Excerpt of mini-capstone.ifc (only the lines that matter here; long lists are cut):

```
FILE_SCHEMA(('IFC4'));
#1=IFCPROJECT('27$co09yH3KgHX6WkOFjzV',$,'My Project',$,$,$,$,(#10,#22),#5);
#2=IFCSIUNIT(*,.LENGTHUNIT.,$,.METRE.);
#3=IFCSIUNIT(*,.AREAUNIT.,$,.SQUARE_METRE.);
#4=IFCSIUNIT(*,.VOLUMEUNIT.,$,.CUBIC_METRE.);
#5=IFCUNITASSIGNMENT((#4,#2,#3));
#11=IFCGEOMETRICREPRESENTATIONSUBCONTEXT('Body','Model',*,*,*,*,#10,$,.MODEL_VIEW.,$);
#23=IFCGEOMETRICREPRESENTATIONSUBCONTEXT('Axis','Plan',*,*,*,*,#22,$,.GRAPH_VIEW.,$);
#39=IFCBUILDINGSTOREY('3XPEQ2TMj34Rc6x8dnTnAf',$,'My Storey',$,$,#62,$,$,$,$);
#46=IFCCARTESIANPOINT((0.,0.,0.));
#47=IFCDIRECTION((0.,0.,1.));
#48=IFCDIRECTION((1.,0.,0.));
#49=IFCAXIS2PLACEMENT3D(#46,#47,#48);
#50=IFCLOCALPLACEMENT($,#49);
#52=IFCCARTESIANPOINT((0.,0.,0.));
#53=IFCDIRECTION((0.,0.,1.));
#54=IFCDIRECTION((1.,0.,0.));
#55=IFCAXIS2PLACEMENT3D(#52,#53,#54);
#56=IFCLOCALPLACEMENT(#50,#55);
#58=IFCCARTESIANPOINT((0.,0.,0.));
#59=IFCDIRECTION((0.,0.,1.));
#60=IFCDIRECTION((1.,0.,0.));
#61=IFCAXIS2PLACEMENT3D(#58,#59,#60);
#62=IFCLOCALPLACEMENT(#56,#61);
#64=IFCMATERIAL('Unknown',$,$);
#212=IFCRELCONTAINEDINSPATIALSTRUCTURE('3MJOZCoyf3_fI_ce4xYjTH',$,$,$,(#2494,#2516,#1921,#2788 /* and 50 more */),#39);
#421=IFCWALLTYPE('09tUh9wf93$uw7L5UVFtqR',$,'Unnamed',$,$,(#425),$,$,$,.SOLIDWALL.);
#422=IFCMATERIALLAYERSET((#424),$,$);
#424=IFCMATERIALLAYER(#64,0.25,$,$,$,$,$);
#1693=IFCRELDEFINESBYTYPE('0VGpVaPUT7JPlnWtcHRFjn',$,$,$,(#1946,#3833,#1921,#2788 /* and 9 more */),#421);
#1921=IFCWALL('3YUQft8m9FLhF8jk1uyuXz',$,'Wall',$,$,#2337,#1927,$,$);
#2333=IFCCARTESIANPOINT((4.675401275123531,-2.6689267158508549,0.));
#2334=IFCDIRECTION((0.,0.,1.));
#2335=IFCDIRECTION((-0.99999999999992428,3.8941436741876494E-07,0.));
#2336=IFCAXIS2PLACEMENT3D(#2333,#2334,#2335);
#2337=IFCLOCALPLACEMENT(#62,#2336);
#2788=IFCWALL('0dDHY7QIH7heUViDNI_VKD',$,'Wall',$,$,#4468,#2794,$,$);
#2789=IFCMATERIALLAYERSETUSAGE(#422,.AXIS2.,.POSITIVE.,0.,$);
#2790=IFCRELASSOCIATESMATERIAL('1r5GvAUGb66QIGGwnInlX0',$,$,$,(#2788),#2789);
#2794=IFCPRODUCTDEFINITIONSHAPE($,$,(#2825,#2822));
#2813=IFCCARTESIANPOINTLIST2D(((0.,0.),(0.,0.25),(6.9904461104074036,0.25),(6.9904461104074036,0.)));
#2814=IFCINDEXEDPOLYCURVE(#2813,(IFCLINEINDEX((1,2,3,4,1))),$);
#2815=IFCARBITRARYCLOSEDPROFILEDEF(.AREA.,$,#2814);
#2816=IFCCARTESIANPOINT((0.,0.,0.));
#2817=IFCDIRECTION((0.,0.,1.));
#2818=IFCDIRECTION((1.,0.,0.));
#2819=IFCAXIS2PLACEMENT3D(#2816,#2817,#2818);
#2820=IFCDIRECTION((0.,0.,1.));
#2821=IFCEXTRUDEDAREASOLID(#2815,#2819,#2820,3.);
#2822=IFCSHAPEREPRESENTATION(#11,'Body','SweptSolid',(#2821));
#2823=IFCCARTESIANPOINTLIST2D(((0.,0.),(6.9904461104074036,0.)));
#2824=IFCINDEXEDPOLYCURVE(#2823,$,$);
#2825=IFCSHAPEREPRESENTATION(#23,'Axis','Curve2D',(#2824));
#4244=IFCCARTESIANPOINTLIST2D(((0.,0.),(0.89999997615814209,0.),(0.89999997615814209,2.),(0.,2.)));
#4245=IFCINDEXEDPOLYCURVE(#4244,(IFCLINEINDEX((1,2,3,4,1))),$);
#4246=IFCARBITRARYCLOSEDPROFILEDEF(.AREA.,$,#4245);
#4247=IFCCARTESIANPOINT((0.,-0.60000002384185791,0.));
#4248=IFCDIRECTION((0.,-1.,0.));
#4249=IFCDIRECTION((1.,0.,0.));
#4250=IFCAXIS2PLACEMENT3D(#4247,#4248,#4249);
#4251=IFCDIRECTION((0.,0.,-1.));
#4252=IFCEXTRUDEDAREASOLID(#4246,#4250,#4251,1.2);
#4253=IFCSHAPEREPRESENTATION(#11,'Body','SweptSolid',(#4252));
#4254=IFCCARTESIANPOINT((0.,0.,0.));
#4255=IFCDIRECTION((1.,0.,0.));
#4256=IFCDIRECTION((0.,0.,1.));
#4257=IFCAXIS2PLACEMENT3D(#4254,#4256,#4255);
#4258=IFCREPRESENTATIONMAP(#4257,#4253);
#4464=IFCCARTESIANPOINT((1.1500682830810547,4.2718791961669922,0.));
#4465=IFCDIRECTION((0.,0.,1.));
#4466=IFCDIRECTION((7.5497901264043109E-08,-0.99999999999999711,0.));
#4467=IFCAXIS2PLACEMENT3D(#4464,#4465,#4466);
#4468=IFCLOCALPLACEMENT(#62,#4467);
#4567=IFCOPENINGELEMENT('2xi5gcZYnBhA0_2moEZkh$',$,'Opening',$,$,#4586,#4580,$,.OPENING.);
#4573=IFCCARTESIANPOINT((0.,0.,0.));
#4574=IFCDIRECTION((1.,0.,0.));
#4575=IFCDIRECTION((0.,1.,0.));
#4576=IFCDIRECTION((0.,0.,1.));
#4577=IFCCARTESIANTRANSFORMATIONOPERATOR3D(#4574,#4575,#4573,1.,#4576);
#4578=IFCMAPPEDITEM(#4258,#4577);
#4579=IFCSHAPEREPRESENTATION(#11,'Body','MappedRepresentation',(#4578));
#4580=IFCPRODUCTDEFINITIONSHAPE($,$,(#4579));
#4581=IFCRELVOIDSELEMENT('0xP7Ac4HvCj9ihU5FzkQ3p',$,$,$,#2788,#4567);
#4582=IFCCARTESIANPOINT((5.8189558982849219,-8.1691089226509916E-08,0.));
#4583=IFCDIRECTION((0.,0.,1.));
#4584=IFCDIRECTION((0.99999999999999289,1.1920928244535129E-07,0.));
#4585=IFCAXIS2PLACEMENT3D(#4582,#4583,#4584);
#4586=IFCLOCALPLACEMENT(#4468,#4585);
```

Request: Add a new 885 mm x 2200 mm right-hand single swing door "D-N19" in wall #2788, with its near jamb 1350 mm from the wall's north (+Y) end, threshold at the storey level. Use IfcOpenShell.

```python
import numpy as np
import ifcopenshell
import ifcopenshell.api.feature
import ifcopenshell.api.geometry
import ifcopenshell.api.root
import ifcopenshell.api.spatial
import ifcopenshell.geom
import ifcopenshell.util.element
import ifcopenshell.util.placement
import ifcopenshell.util.representation
import ifcopenshell.util.shape
import ifcopenshell.util.unit

model = ifcopenshell.open("mini-capstone.ifc")
unit_scale = ifcopenshell.util.unit.calculate_unit_scale(model)
settings = ifcopenshell.geom.settings()


def volume(element):
    """Net volume in cubic metres, openings subtracted."""
    shape = ifcopenshell.geom.create_shape(settings, element)
    return ifcopenshell.util.shape.get_volume(shape.geometry)


wall = model.by_guid("0dDHY7QIH7heUViDNI_VKD")
storey = ifcopenshell.util.element.get_container(wall, ifc_class="IfcBuildingStorey")
context = ifcopenshell.util.representation.get_context(model, "Model", "Body", "MODEL_VIEW")
before = volume(wall)

width, height, from_end, sill = 0.885, 2.2, 1.35, 0.0  # metres

# The wall runs along its own X axis, and the end named is its -X end.
wall_shape = ifcopenshell.geom.create_shape(settings, wall)
x, y, z = ifcopenshell.util.shape.get_vertices(wall_shape.geometry).T
start = x.min() + from_end
face, thickness = float(y.min()), float(y.max() - y.min())
wall_matrix = ifcopenshell.util.placement.get_local_placement(wall.ObjectPlacement)
level = ifcopenshell.util.placement.get_local_placement(storey.ObjectPlacement)[2, 3]


def in_wall(x, y):
    """Placement at x, y metres in the wall's axes, at sill height."""
    matrix = wall_matrix.copy()
    matrix[:, 3] = wall_matrix @ np.array([x / unit_scale, y / unit_scale, 0.0, 1.0])
    matrix[2, 3] = level + sill / unit_scale
    return matrix


# Opening: a box that overshoots both wall faces by 50 mm.
opening = ifcopenshell.api.root.create_entity(model, ifc_class="IfcOpeningElement", predefined_type="OPENING")
box = ifcopenshell.api.geometry.add_wall_representation(
    model, context=context, length=width, height=height, thickness=thickness + 0.1
)
ifcopenshell.api.geometry.assign_representation(model, product=opening, representation=box)
ifcopenshell.api.geometry.edit_object_placement(model, product=opening, matrix=in_wall(start, face - 0.05), is_si=False)
ifcopenshell.api.feature.add_feature(model, feature=opening, element=wall)

door = ifcopenshell.api.root.create_entity(model, ifc_class="IfcDoor", name="D-N19", predefined_type="DOOR")
door.OverallWidth, door.OverallHeight = width / unit_scale, height / unit_scale
door.OperationType = "SINGLE_SWING_RIGHT"
body = ifcopenshell.api.geometry.add_door_representation(
    model,
    context=context,
    overall_width=door.OverallWidth,
    overall_height=door.OverallHeight,
    operation_type="SINGLE_SWING_RIGHT",
    lining_properties={"LiningDepth": thickness / unit_scale, "ThresholdDepth": thickness / unit_scale},
)
ifcopenshell.api.geometry.assign_representation(model, product=door, representation=body)
ifcopenshell.api.spatial.assign_container(model, products=[door], relating_structure=storey)
ifcopenshell.api.feature.add_filling(model, opening=opening, element=door)

# The lining spans the wall, so the door starts at the wall face.
ifcopenshell.api.geometry.edit_object_placement(model, product=door, matrix=in_wall(start, face), is_si=False)

after = volume(wall)

print(f"wall volume {before:.3f} -> {after:.3f} m3")

model.write("mini-capstone-out.ifc")
```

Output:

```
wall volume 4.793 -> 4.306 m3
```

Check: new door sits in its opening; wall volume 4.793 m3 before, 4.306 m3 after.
